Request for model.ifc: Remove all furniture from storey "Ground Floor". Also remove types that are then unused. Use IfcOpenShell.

First a look at what the model holds.

```python
import ifcopenshell
import ifcopenshell.util.element

model = ifcopenshell.open("model.ifc")
print(model.schema)
storey = next(s for s in model.by_type("IfcBuildingStorey") if s.Name == "Ground Floor")
furniture = [e for e in ifcopenshell.util.element.get_decomposition(storey) if e.is_a("IfcFurnishingElement")]
seen = {}
for e in furniture:
    element_type = ifcopenshell.util.element.get_type(e)
    name = element_type.Name if element_type not in (None, e) else None
    seen[name] = seen.get(name, 0) + 1
for name, count in sorted(seen.items(), key=str):
    print(count, "x", name)
```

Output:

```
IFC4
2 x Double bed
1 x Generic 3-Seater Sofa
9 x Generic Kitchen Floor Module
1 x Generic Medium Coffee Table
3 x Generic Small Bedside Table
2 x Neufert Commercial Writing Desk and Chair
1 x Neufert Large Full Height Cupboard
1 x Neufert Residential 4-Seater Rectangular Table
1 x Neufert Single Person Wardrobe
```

```python
import ifcopenshell
import ifcopenshell.api.root
import ifcopenshell.util.element

model = ifcopenshell.open("model.ifc")

storey = next(s for s in model.by_type("IfcBuildingStorey") if s.Name == "Ground Floor")
furniture = [e for e in ifcopenshell.util.element.get_decomposition(storey) if e.is_a("IfcFurnishingElement")]
types = {ifcopenshell.util.element.get_type(e) for e in furniture} - {None, *furniture}

for e in furniture:
    ifcopenshell.api.root.remove_product(model, product=e)
print(len(furniture), "removed")

unused = [t for t in types if not ifcopenshell.util.element.get_types(t)]
for t in unused:
    ifcopenshell.api.root.remove_product(model, product=t)
print(len(unused), "unused types removed")

model.write("model_updated.ifc")
```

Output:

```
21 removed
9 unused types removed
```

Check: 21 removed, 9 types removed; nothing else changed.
